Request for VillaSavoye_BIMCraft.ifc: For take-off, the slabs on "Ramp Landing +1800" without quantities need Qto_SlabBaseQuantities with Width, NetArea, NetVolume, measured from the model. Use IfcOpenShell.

First a look at what the model holds.

```python
import ifcopenshell
import ifcopenshell.util.element
import ifcopenshell.util.unit

model = ifcopenshell.open("VillaSavoye_BIMCraft.ifc")
print(model.schema)
for unit_type in ("LENGTHUNIT", "AREAUNIT", "VOLUMEUNIT"):
    print(unit_type, ifcopenshell.util.unit.calculate_unit_scale(model, unit_type))
storey = next(s for s in model.by_type("IfcBuildingStorey") if s.Name == "Ramp Landing +1800")
slabs = [e for e in ifcopenshell.util.element.get_decomposition(storey) if e.is_a("IfcSlab")]
for e in sorted(slabs, key=lambda e: e.id()):
    print(e.id(), e.is_a(), e.Name, list(ifcopenshell.util.element.get_psets(e, qtos_only=True)), sep=" | ")
```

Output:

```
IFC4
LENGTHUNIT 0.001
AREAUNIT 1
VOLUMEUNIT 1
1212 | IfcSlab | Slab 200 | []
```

```python
import ifcopenshell
import ifcopenshell.api.pset
import ifcopenshell.geom
import ifcopenshell.util.element
import ifcopenshell.util.shape
import ifcopenshell.util.unit

model = ifcopenshell.open("VillaSavoye_BIMCraft.ifc")
unit_scale = ifcopenshell.util.unit.calculate_unit_scale(model)
area_scale = ifcopenshell.util.unit.calculate_unit_scale(model, "AREAUNIT")
volume_scale = ifcopenshell.util.unit.calculate_unit_scale(model, "VOLUMEUNIT")
settings = ifcopenshell.geom.settings()

storey = next(s for s in model.by_type("IfcBuildingStorey") if s.Name == "Ramp Landing +1800")
slabs = [e for e in ifcopenshell.util.element.get_decomposition(storey) if e.is_a("IfcSlab")]

for e in sorted(slabs, key=lambda e: e.id()):
    if ifcopenshell.util.element.get_psets(e, qtos_only=True, should_inherit=False):
        continue
    # Geometry comes back in metres, in the element's own axes.
    shape = ifcopenshell.geom.create_shape(settings, e)
    values = {
        "Width": ifcopenshell.util.shape.get_z(shape.geometry) / unit_scale,
        "NetArea": ifcopenshell.util.shape.get_footprint_area(shape.geometry) / area_scale,
        "NetVolume": ifcopenshell.util.shape.get_volume(shape.geometry) / volume_scale,
    }
    qto = ifcopenshell.api.pset.add_qto(model, product=e, name="Qto_SlabBaseQuantities")
    ifcopenshell.api.pset.edit_qto(model, qto=qto, properties=values)
    print(e.id(), {k: round(v, 3) for k, v in values.items()})

model.write("VillaSavoye_BIMCraft_edited.ifc")
```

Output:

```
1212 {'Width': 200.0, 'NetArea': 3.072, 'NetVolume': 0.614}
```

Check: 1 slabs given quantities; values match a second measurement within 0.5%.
